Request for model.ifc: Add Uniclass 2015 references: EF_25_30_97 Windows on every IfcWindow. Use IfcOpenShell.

First a look at what the model holds.

```python
import ifcopenshell

model = ifcopenshell.open("model.ifc")
print(model.schema)
print("classifications:", [c.Name for c in model.by_type("IfcClassification")])
for ifc_class in ("IfcDoor", "IfcRoof", "IfcStair", "IfcWall", "IfcWindow"):
    print(ifc_class, len(model.by_type(ifc_class)))
```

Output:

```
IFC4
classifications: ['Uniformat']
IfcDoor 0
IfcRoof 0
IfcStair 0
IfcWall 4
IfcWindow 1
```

```python
import ifcopenshell
import ifcopenshell.api.classification

model = ifcopenshell.open("model.ifc")

system = ifcopenshell.api.classification.add_classification(model, classification="Uniclass 2015")

codes = {
    "IfcWindow": ("EF_25_30_97", "Windows"),
}
for ifc_class, (code, name) in codes.items():
    products = model.by_type(ifc_class)
    ifcopenshell.api.classification.add_reference(
        model, products=products, classification=system, identification=code, name=name
    )
    print(code, len(products))

model.write("model_updated.ifc")
```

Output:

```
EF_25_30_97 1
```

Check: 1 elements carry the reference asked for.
